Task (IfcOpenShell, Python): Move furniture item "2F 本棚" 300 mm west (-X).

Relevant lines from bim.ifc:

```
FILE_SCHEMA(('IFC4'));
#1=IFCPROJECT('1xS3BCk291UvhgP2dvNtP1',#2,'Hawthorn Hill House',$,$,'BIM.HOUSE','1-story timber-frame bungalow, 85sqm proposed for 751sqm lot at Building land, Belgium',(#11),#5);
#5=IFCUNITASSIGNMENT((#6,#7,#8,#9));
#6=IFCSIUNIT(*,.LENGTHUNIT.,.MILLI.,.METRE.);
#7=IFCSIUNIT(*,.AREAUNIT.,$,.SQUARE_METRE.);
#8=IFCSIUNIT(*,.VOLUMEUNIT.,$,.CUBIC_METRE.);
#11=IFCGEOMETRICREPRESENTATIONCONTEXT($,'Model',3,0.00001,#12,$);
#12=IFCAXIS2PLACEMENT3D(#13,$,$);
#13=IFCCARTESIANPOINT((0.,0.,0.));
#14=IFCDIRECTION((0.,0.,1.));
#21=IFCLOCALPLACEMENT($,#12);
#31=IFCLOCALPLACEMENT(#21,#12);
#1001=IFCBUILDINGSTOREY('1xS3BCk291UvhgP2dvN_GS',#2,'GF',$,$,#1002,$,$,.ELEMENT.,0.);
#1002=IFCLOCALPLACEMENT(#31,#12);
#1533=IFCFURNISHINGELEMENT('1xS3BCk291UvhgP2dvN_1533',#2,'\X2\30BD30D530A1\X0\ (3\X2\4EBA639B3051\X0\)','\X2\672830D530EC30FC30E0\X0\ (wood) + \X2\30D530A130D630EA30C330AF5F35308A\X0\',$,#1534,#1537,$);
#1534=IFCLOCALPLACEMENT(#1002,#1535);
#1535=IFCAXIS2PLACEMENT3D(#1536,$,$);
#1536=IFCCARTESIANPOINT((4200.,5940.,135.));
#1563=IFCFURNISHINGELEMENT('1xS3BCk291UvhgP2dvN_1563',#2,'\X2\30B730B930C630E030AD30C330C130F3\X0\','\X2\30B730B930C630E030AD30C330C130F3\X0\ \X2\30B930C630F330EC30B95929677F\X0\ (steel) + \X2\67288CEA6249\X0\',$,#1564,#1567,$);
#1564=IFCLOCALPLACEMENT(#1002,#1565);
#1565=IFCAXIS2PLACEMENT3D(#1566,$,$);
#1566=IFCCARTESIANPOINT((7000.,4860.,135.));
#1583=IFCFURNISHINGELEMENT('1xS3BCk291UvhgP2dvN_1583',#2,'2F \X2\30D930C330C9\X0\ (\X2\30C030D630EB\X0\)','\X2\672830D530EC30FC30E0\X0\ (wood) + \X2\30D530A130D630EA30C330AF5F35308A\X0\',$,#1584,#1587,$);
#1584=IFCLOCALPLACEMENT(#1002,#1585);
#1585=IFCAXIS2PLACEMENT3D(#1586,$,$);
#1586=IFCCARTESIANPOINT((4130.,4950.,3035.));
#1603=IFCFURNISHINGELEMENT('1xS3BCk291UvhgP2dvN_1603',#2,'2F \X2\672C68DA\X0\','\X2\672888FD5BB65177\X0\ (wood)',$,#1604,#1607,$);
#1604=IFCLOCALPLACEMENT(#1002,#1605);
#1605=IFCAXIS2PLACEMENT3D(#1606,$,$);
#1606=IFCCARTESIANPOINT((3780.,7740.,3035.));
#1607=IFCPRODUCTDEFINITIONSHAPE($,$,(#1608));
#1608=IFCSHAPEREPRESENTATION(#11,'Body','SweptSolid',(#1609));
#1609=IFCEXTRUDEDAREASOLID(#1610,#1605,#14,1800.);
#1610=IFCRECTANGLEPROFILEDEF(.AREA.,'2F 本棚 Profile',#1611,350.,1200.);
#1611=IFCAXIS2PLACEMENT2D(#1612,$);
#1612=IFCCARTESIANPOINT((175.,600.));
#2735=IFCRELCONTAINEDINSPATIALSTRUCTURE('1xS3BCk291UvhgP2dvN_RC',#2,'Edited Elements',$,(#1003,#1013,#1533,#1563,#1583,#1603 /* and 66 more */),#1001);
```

```python
import ifcopenshell
import ifcopenshell.api.geometry
import ifcopenshell.util.placement
import ifcopenshell.util.unit

model = ifcopenshell.open("bim.ifc")
unit_scale = ifcopenshell.util.unit.calculate_unit_scale(model)

item = model.by_guid("1xS3BCk291UvhgP2dvN_1603")
matrix = ifcopenshell.util.placement.get_local_placement(item.ObjectPlacement)
matrix[0, 3] -= 0.3 / unit_scale
ifcopenshell.api.geometry.edit_object_placement(model, product=item, matrix=matrix, is_si=False)

print(ifcopenshell.util.placement.get_local_placement(item.ObjectPlacement).round(3) + 0.0)

model.write("bim_edited.ifc")
```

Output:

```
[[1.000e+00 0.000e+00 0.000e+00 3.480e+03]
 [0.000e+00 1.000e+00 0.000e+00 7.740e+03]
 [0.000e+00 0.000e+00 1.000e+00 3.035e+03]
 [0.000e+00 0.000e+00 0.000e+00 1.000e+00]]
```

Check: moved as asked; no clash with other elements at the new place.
